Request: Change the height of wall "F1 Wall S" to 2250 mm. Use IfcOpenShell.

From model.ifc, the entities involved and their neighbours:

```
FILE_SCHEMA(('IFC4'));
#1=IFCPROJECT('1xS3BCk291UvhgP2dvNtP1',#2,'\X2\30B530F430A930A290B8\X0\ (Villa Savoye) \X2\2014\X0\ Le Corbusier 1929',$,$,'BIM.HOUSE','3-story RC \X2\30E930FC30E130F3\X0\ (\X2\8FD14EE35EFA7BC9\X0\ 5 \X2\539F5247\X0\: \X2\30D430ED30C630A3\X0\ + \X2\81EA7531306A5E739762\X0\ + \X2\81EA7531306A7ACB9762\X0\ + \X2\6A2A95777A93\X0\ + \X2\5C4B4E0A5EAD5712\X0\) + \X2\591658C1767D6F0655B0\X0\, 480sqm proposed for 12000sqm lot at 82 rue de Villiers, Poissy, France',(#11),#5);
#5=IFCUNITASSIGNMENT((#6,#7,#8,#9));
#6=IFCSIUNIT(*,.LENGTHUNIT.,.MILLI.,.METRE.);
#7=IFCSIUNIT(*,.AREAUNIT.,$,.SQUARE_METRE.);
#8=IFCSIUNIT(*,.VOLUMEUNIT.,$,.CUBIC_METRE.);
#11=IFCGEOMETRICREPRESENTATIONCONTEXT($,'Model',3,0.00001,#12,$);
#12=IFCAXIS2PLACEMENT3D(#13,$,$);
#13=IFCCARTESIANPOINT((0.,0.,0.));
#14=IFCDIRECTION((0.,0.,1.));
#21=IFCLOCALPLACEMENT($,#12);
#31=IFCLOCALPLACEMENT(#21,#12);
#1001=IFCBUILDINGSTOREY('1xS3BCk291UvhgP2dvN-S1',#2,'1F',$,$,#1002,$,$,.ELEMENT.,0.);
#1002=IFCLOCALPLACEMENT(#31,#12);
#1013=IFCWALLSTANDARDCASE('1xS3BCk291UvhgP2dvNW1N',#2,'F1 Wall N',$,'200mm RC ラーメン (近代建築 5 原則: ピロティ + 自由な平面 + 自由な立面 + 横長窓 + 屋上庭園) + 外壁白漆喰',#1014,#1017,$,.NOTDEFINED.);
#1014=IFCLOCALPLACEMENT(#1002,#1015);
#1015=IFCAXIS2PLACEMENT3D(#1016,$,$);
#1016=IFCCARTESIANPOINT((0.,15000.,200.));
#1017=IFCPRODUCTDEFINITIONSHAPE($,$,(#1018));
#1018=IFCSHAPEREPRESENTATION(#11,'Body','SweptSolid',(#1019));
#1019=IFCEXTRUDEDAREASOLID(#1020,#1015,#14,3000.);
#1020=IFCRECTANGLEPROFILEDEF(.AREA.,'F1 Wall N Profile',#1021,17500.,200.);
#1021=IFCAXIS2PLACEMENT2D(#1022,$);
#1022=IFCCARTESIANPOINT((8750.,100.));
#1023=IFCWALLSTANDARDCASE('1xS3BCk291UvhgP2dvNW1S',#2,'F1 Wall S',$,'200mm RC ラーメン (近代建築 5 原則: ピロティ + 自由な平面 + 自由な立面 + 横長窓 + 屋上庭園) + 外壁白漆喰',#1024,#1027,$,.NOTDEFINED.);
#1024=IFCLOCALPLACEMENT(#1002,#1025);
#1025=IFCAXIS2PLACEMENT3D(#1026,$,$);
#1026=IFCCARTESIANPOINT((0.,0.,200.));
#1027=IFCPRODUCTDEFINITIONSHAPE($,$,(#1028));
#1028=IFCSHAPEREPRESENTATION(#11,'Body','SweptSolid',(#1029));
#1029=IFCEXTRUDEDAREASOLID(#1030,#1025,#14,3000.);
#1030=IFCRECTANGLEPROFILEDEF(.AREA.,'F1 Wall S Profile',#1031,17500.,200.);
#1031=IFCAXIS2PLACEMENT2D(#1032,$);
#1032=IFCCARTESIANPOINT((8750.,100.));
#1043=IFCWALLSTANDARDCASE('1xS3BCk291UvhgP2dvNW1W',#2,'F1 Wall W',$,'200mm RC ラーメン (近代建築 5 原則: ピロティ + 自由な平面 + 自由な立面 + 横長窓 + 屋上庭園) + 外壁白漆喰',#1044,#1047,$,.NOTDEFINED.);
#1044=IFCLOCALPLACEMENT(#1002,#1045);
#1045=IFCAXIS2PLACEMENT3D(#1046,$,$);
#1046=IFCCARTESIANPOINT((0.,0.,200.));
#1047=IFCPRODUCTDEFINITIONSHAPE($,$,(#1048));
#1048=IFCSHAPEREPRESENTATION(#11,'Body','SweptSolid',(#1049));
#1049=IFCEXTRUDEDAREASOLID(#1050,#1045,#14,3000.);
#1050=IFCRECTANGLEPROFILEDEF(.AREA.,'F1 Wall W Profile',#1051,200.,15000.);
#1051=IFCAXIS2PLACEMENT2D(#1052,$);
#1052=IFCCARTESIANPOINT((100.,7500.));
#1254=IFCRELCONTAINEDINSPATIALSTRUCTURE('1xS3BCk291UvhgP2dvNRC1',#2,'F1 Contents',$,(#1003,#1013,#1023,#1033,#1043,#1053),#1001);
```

```python
import ifcopenshell
import ifcopenshell.geom
import ifcopenshell.util.shape
import ifcopenshell.util.unit

model = ifcopenshell.open("model.ifc")
unit_scale = ifcopenshell.util.unit.calculate_unit_scale(model)
settings = ifcopenshell.geom.settings()


def volume(element):
    """Net volume in cubic metres, openings subtracted."""
    shape = ifcopenshell.geom.create_shape(settings, element)
    return ifcopenshell.util.shape.get_volume(shape.geometry)


wall = model.by_guid("1xS3BCk291UvhgP2dvNW1S")
before = volume(wall)

body = next(r for r in wall.Representation.Representations if r.RepresentationIdentifier == "Body")
solid = body.Items[0]
old_height = solid.Depth
solid.Depth = 2.25 / unit_scale
after = volume(wall)

print(f"height {old_height:g} -> {solid.Depth:g}, volume {before:.3f} -> {after:.3f} m3")

model.write("model_rev.ifc")
```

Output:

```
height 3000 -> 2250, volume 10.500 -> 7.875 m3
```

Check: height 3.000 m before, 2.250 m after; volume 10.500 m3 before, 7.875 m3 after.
